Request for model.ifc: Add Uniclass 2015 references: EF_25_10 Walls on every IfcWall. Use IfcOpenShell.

First a look at what the model holds.

```python
import ifcopenshell

model = ifcopenshell.open("model.ifc")
print(model.schema)
print("classifications:", [c.Name for c in model.by_type("IfcClassification")])
for ifc_class in ("IfcDoor", "IfcRoof", "IfcStair", "IfcWall", "IfcWindow"):
    print(ifc_class, len(model.by_type(ifc_class)))
```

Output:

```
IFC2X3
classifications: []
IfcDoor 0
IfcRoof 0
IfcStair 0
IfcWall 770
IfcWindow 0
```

```python
import ifcopenshell
import ifcopenshell.api.classification

model = ifcopenshell.open("model.ifc")

# IFC2X3 requires Source and Edition and has no link from the project to the system.
system = model.create_entity("IfcClassification", Source="NBS", Edition="2015", Name="Uniclass 2015")

codes = {
    "IfcWall": ("EF_25_10", "Walls"),
}
for ifc_class, (code, name) in codes.items():
    products = model.by_type(ifc_class)
    ifcopenshell.api.classification.add_reference(
        model, products=products, classification=system, identification=code, name=name
    )
    print(code, len(products))

model.write("model_v2.ifc")
```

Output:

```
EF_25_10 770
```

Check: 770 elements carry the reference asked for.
